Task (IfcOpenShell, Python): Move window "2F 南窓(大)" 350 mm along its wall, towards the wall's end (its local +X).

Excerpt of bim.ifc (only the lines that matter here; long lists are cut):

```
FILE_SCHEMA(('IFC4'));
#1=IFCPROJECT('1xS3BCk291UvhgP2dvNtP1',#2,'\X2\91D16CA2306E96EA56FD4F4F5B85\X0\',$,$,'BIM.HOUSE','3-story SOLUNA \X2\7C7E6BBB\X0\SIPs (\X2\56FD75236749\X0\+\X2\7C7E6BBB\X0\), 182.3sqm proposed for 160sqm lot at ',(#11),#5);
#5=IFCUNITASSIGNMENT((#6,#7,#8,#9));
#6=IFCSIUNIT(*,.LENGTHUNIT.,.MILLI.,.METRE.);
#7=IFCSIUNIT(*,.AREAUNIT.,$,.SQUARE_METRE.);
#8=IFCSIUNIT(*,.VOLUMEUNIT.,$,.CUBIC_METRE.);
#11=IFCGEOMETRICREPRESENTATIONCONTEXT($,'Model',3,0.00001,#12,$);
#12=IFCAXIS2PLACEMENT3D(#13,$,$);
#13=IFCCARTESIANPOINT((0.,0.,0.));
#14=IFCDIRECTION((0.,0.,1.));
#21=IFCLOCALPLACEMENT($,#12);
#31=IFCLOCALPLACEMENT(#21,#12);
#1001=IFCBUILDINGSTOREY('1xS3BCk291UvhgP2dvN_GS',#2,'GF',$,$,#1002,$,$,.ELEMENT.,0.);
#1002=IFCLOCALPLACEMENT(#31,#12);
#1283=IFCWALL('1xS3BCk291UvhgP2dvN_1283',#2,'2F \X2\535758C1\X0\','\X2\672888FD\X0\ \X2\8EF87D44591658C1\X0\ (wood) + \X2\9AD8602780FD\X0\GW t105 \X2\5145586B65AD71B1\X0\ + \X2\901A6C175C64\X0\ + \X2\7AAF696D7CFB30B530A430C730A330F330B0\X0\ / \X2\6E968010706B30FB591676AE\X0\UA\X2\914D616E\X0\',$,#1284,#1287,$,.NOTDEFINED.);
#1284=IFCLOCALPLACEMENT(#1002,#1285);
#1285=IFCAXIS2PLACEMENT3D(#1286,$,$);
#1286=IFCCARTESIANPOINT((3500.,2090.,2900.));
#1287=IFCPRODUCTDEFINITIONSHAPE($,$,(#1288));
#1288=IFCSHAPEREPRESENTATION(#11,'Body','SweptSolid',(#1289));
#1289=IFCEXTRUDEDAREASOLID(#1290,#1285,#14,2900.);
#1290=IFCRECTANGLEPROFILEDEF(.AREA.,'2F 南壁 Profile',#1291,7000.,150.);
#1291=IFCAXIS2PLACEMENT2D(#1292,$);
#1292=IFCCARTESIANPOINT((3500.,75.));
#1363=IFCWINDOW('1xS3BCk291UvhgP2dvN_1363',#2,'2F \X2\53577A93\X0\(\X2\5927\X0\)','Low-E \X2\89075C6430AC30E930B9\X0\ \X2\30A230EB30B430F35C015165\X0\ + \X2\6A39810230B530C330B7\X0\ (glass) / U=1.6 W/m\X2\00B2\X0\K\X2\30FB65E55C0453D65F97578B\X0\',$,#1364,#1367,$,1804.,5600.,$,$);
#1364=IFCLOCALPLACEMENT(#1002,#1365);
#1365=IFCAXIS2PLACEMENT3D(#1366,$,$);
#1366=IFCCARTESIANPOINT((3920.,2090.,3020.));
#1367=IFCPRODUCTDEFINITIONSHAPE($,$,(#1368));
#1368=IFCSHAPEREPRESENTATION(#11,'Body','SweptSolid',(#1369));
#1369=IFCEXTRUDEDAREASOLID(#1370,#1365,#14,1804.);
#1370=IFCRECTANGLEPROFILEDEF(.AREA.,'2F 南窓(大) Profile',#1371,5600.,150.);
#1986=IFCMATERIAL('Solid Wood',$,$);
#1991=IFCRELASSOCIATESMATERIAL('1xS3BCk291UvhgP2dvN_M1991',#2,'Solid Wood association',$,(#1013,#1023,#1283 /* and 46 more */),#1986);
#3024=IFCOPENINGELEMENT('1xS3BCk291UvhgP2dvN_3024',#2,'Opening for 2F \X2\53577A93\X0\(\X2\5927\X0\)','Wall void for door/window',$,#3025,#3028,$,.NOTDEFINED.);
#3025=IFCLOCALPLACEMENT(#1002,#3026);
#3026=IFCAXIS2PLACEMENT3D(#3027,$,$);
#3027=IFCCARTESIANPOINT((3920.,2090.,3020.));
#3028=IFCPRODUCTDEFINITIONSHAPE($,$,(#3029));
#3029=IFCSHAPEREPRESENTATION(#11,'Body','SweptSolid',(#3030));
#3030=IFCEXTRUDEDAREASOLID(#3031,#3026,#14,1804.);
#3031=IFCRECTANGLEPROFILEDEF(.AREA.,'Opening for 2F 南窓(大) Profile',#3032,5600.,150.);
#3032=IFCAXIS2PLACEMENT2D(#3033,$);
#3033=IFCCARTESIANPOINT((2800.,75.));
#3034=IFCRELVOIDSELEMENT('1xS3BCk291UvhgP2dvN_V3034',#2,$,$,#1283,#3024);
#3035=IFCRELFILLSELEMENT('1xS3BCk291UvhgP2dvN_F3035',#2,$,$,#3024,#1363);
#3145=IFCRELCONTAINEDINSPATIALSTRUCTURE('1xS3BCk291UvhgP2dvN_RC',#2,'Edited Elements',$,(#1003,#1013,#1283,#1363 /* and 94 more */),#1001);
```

```python
import ifcopenshell
import ifcopenshell.api.geometry
import ifcopenshell.util.placement
import ifcopenshell.util.unit

model = ifcopenshell.open("bim.ifc")
unit_scale = ifcopenshell.util.unit.calculate_unit_scale(model)

window = model.by_guid("1xS3BCk291UvhgP2dvN_1363")
opening = window.FillsVoids[0].RelatingOpeningElement
wall = opening.VoidsElements[0].RelatingBuildingElement

wall_matrix = ifcopenshell.util.placement.get_local_placement(wall.ObjectPlacement)
shift = wall_matrix[:3, 0] * 0.35 / unit_scale
before = ifcopenshell.util.placement.get_local_placement(window.ObjectPlacement)[:3, 3].copy()

# The window is not placed relative to its opening, so move both.
for product in (opening, window):
    matrix = ifcopenshell.util.placement.get_local_placement(product.ObjectPlacement)
    matrix[:3, 3] += shift
    ifcopenshell.api.geometry.edit_object_placement(model, product=product, matrix=matrix, is_si=False)

after = ifcopenshell.util.placement.get_local_placement(window.ObjectPlacement)[:3, 3]
print("window moved by", (after - before).round(3) + 0.0)

model.write("bim_edited.ifc")
```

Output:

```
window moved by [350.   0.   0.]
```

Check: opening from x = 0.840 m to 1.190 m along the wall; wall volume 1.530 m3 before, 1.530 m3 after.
